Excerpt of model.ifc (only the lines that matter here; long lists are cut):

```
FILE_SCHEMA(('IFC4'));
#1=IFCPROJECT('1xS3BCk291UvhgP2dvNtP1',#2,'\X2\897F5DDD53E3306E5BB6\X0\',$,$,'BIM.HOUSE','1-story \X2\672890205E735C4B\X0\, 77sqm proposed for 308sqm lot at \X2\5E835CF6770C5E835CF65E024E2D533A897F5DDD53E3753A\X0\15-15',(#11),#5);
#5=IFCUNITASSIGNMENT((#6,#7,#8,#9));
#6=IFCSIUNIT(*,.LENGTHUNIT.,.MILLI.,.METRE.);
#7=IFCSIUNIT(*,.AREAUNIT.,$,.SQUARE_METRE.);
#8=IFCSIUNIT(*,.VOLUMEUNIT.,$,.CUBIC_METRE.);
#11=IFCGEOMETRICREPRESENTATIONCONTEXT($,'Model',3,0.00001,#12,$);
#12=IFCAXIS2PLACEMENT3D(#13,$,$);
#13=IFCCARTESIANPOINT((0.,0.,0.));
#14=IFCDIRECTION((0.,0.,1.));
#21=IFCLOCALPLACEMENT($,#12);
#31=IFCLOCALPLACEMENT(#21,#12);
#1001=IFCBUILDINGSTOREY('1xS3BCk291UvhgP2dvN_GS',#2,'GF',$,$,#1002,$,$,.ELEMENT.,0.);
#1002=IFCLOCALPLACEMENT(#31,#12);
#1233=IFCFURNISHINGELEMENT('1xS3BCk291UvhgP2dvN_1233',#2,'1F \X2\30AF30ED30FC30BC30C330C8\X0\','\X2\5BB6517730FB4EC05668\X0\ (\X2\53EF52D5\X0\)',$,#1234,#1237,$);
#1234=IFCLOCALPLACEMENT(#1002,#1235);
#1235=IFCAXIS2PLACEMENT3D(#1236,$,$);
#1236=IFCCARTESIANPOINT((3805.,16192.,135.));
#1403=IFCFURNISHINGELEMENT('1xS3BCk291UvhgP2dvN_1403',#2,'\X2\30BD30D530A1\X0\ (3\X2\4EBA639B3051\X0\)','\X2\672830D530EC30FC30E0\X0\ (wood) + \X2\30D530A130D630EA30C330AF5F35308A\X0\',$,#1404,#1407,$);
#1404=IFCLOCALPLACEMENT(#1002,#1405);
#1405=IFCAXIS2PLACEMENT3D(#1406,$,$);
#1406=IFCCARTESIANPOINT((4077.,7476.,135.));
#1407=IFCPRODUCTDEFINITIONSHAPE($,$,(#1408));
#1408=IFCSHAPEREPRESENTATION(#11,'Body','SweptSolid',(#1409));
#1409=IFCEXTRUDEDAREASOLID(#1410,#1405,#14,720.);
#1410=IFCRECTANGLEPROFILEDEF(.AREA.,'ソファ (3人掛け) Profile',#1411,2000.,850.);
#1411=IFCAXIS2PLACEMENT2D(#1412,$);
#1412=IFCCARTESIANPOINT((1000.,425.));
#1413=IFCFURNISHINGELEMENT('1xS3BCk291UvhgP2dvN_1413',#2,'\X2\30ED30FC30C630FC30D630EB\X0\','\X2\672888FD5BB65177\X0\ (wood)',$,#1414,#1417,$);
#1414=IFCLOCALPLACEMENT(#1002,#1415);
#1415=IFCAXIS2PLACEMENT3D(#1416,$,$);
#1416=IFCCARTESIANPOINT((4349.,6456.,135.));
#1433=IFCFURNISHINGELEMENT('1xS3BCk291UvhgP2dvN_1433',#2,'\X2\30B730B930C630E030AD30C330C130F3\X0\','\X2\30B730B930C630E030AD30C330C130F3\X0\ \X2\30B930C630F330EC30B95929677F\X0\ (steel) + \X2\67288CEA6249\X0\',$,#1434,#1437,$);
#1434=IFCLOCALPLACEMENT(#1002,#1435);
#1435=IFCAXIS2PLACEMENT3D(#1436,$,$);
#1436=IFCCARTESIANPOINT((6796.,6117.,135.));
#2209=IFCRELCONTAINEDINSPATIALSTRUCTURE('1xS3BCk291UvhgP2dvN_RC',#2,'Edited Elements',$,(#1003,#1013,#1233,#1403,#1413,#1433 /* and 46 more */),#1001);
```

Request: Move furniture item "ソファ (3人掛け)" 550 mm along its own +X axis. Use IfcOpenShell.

```python
import ifcopenshell
import ifcopenshell.api.geometry
import ifcopenshell.util.placement

model = ifcopenshell.open("model.ifc")

item = model.by_id(1403)
matrix = ifcopenshell.util.placement.get_local_placement(item.ObjectPlacement)
matrix[:3, 3] += matrix[:3, 0] * 550.0
ifcopenshell.api.geometry.edit_object_placement(model, product=item, matrix=matrix, is_si=False)

print(ifcopenshell.util.placement.get_local_placement(item.ObjectPlacement).round(3) + 0.0)

model.write("model_edited.ifc")
```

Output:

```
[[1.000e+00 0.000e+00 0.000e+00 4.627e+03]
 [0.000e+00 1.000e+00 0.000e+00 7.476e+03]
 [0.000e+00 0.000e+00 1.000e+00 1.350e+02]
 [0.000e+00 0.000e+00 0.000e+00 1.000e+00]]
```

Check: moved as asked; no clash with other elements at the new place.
